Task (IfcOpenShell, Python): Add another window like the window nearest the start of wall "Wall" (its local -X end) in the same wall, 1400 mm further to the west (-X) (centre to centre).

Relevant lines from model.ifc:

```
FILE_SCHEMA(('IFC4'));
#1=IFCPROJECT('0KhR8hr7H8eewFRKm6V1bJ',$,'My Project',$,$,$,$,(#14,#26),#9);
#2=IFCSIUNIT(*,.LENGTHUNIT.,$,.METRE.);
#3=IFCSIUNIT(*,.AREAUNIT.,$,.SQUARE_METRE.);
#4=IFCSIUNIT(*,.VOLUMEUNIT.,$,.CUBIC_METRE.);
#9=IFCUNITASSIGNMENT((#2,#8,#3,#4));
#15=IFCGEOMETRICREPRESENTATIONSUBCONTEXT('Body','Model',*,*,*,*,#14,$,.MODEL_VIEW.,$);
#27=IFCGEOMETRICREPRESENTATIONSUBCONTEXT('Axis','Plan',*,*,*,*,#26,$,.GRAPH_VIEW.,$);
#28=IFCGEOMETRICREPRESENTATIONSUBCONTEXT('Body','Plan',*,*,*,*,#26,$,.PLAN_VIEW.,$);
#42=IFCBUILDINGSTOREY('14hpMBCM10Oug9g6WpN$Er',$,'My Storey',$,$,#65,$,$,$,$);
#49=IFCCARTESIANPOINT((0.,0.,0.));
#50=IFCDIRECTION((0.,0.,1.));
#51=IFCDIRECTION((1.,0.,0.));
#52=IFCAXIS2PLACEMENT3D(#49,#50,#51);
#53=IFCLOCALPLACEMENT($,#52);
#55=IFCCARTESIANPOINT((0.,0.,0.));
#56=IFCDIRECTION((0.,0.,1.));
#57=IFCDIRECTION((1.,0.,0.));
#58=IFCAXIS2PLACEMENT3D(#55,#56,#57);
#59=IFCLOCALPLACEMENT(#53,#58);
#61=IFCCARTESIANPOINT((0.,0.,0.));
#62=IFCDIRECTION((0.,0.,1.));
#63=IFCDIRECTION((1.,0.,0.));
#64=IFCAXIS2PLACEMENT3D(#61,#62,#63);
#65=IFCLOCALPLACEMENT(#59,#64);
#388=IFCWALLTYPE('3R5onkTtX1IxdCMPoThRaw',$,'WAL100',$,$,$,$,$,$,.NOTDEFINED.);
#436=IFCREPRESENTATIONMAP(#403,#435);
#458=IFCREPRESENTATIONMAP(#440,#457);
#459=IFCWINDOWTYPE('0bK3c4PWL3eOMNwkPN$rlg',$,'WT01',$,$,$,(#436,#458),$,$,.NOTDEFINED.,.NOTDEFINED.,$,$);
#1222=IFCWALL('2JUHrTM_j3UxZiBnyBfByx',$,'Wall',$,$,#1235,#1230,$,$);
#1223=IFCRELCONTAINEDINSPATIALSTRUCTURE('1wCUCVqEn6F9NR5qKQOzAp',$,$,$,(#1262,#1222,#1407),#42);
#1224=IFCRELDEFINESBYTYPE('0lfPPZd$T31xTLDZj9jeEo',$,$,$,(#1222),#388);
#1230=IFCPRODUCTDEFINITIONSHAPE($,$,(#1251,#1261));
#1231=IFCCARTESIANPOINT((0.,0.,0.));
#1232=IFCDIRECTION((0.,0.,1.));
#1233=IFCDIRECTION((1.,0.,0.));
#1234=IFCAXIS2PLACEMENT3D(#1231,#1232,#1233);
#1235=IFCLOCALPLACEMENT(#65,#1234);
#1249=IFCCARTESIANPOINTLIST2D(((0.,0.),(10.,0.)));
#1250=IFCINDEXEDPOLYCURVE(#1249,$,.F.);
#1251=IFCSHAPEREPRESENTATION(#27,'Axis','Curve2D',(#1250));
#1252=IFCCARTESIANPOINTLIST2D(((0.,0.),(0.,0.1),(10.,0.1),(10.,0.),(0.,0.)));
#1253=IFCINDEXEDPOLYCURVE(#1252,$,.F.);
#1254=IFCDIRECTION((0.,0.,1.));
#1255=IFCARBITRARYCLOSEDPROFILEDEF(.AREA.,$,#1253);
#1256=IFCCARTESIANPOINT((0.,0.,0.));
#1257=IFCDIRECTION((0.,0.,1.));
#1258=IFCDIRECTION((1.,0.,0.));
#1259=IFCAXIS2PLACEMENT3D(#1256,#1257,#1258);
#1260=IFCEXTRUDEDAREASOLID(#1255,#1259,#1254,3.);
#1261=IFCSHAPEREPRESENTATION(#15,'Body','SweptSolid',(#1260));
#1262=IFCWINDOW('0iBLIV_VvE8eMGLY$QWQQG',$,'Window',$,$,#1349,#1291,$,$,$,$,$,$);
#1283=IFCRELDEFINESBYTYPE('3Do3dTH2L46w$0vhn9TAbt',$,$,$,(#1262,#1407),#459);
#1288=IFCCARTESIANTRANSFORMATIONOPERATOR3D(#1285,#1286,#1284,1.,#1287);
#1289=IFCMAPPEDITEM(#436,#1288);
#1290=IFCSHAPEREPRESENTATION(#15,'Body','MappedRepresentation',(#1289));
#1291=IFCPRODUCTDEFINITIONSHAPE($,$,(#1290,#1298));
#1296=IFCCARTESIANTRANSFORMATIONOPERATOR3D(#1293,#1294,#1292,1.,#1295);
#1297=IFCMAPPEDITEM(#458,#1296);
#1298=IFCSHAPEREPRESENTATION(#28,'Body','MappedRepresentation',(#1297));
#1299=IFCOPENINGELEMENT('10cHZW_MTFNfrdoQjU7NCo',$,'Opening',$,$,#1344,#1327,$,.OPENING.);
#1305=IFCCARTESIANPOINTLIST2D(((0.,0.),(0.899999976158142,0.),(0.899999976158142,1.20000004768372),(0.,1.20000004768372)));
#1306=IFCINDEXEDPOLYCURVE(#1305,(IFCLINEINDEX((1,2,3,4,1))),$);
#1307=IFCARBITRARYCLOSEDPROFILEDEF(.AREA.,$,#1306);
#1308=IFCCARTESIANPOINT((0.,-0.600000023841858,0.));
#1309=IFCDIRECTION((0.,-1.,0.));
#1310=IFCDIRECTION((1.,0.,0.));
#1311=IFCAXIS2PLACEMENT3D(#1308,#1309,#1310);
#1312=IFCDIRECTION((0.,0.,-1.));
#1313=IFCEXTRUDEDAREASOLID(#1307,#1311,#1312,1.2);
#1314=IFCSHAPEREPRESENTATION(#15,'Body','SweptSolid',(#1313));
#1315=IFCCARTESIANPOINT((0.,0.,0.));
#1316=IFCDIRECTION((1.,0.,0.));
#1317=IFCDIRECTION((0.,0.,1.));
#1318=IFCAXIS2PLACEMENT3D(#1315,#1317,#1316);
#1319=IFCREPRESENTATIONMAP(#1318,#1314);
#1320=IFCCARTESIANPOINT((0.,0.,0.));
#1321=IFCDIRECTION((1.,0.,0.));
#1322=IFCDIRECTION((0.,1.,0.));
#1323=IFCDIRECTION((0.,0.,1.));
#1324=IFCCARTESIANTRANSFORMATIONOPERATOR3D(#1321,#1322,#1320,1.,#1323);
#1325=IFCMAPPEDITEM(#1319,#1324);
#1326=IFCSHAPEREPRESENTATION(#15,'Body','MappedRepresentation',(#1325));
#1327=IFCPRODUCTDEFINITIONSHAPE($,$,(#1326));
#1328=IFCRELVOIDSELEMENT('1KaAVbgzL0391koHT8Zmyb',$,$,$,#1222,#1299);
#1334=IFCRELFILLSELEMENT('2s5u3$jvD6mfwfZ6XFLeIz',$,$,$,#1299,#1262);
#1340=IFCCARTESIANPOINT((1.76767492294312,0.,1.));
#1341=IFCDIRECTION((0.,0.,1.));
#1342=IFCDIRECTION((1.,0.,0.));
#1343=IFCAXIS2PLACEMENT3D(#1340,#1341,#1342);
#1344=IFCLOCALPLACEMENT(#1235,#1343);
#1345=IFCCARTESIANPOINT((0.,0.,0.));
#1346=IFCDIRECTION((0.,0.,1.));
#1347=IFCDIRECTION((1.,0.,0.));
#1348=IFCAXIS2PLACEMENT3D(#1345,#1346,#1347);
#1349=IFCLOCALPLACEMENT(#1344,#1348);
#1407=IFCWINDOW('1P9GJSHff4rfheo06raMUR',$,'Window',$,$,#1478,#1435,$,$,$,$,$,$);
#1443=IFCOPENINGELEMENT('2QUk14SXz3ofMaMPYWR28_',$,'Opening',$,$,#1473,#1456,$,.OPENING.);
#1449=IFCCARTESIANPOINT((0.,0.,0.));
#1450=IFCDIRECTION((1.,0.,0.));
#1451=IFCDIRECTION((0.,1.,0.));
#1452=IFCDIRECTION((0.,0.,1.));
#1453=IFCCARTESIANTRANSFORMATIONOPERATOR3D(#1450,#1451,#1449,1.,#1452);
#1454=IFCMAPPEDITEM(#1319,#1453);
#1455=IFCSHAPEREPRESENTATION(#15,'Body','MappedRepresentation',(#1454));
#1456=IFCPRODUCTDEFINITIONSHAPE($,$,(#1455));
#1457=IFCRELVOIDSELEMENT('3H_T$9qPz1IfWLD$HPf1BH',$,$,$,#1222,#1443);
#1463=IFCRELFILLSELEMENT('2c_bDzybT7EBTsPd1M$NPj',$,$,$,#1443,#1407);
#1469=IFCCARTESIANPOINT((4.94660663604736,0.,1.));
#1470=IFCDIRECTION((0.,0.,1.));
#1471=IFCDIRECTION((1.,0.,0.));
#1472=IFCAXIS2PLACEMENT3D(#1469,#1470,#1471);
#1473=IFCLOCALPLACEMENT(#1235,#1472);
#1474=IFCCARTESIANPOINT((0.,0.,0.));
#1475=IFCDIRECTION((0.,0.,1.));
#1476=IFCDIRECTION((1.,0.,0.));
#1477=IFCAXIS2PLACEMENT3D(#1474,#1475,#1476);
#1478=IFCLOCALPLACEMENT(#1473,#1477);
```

```python
import ifcopenshell
import ifcopenshell.api.feature
import ifcopenshell.api.geometry
import ifcopenshell.api.root
import ifcopenshell.geom
import ifcopenshell.util.element
import ifcopenshell.util.placement
import ifcopenshell.util.shape
import ifcopenshell.util.unit

model = ifcopenshell.open("model.ifc")
unit_scale = ifcopenshell.util.unit.calculate_unit_scale(model)
settings = ifcopenshell.geom.settings()


def volume(element):
    """Net volume in cubic metres, openings subtracted."""
    shape = ifcopenshell.geom.create_shape(settings, element)
    return ifcopenshell.util.shape.get_volume(shape.geometry)


window = model.by_id(1262)
opening = window.FillsVoids[0].RelatingOpeningElement
wall = opening.VoidsElements[0].RelatingBuildingElement
before = volume(wall)
shift = ifcopenshell.util.placement.get_local_placement(wall.ObjectPlacement)[:3, 0] * -1.4 / unit_scale

# copy_class copies the void relationship, type, container and properties, but no geometry.
new_opening = ifcopenshell.api.root.copy_class(model, product=opening)
new_opening.Representation = ifcopenshell.util.element.copy_deep(
    model, opening.Representation, exclude=["IfcGeometricRepresentationContext", "IfcRepresentationMap"]
)
new_window = ifcopenshell.api.root.copy_class(model, product=window)
new_window.Representation = ifcopenshell.util.element.copy_deep(
    model, window.Representation, exclude=["IfcGeometricRepresentationContext", "IfcRepresentationMap"]
)
ifcopenshell.api.feature.add_filling(model, opening=new_opening, element=new_window)

for old, new in ((opening, new_opening), (window, new_window)):
    matrix = ifcopenshell.util.placement.get_local_placement(old.ObjectPlacement)
    matrix[:3, 3] += shift
    ifcopenshell.api.geometry.edit_object_placement(model, product=new, matrix=matrix, is_si=False)

after = volume(wall)

print(f"wall volume {before:.3f} -> {after:.3f} m3")

model.write("model_v2.ifc")
```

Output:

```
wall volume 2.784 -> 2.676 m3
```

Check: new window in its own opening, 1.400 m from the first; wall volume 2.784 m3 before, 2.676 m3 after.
